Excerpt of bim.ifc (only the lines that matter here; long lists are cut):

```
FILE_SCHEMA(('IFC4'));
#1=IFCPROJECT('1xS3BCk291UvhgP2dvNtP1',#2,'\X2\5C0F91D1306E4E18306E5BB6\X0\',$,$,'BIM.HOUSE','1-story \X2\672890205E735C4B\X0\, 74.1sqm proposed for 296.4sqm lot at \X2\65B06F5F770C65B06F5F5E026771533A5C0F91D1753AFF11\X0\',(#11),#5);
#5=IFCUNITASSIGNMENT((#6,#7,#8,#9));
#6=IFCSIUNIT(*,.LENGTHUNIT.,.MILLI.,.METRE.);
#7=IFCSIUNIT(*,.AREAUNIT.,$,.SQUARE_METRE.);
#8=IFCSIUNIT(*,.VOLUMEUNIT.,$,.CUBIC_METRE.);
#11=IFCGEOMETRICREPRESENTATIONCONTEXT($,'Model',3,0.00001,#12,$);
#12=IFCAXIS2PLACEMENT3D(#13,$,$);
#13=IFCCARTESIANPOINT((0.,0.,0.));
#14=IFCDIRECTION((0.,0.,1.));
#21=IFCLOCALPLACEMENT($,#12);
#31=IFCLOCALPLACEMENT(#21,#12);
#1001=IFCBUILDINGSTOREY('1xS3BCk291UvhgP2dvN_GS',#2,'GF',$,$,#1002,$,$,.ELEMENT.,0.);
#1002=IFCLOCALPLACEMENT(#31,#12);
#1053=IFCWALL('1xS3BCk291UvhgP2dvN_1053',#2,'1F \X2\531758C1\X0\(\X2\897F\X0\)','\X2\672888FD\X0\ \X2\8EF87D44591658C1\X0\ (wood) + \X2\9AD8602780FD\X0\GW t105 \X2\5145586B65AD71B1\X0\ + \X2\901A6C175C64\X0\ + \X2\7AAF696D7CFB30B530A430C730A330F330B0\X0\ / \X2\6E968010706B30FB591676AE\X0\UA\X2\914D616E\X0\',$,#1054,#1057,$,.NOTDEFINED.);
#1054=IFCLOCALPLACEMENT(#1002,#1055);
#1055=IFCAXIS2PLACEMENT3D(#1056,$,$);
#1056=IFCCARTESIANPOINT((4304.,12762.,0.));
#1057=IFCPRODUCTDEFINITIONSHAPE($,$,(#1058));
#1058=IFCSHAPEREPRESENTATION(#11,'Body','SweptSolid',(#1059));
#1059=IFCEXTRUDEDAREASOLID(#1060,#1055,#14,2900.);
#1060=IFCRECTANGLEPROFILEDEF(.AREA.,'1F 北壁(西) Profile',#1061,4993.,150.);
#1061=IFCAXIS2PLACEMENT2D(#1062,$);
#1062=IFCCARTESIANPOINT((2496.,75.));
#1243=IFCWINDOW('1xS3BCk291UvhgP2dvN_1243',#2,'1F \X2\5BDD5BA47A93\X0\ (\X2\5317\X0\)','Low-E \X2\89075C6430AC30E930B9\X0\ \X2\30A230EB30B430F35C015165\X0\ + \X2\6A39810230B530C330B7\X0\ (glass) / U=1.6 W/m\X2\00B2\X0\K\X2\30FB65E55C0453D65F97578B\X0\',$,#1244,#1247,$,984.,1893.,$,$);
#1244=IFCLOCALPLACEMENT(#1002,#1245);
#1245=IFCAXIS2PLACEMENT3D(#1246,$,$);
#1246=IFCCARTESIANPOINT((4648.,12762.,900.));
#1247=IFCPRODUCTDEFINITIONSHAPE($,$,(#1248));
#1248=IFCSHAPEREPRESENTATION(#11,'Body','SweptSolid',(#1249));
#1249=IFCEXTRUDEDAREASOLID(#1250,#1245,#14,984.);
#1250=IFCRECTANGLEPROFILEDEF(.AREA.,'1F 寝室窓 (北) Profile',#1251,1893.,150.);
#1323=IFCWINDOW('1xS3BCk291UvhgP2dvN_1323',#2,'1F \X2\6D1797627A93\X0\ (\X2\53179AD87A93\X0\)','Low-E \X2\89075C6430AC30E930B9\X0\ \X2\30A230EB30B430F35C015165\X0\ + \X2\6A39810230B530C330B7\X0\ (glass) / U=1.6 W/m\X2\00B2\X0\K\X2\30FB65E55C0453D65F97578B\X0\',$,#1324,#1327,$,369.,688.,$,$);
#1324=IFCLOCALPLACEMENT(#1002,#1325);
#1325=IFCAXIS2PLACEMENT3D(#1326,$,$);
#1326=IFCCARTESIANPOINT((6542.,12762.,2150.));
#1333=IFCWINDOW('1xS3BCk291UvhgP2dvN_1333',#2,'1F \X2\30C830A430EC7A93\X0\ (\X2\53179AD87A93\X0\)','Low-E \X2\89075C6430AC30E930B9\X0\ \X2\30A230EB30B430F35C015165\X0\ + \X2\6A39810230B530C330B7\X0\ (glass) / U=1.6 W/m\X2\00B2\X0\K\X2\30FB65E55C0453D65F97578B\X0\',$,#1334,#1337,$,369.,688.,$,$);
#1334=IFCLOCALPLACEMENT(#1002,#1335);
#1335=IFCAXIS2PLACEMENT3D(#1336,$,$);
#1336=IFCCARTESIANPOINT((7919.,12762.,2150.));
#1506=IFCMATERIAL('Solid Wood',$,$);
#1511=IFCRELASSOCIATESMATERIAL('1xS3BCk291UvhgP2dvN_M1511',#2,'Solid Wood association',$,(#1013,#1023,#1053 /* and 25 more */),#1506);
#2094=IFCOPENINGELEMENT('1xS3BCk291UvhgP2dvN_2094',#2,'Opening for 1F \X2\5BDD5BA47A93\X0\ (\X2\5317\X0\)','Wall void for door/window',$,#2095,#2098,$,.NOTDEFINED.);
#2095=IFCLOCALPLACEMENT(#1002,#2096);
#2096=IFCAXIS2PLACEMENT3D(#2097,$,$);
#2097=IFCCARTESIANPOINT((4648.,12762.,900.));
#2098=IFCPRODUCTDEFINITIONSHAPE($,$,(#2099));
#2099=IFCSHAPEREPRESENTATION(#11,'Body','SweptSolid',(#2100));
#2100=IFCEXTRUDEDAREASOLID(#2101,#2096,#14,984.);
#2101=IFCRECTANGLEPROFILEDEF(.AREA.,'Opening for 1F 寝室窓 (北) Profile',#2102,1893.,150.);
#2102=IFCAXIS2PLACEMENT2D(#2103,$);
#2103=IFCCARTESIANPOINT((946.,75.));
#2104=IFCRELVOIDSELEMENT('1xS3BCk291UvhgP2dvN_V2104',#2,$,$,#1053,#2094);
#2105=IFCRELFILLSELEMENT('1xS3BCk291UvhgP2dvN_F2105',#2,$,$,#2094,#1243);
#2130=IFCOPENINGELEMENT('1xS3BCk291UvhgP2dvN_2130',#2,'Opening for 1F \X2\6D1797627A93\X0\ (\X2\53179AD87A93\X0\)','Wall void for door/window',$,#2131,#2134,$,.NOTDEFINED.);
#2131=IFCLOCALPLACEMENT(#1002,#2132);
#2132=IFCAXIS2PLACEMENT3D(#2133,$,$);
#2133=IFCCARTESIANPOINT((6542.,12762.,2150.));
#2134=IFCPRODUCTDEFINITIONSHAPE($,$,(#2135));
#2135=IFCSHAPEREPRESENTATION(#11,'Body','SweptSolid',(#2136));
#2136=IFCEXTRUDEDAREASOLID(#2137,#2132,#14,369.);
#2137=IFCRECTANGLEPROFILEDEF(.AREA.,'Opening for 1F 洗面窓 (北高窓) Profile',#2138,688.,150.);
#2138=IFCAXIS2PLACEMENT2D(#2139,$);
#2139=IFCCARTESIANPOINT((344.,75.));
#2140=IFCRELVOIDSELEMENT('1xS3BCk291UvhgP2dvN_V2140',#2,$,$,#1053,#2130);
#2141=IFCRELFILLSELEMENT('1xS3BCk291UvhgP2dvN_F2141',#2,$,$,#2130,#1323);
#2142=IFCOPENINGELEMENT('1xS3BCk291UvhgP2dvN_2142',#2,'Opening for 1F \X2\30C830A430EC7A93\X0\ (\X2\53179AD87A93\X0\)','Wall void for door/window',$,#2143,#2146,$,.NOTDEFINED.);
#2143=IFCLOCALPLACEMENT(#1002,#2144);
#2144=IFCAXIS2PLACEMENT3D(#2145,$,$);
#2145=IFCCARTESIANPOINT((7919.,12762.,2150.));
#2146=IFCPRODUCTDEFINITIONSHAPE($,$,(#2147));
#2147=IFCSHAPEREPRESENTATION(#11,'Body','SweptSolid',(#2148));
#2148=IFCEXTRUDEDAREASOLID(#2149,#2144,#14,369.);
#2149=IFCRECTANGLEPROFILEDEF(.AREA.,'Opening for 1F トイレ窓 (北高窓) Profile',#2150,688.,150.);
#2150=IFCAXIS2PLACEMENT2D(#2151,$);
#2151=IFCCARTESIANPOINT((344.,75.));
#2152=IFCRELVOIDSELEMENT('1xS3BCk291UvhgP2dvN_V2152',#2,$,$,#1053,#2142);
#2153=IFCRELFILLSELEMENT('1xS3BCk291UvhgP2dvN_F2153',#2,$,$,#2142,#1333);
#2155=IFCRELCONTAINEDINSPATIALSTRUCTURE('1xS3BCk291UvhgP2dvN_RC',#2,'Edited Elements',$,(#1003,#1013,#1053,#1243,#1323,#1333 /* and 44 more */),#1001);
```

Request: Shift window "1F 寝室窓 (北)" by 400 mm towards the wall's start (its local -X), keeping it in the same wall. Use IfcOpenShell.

```python
import ifcopenshell
import ifcopenshell.api.geometry
import ifcopenshell.util.placement

model = ifcopenshell.open("bim.ifc")

window = model.by_guid("1xS3BCk291UvhgP2dvN_1243")
opening = window.FillsVoids[0].RelatingOpeningElement
wall = opening.VoidsElements[0].RelatingBuildingElement

wall_matrix = ifcopenshell.util.placement.get_local_placement(wall.ObjectPlacement)
shift = wall_matrix[:3, 0] * -400.0
before = ifcopenshell.util.placement.get_local_placement(window.ObjectPlacement)[:3, 3].copy()

# The window is not placed relative to its opening, so move both.
for product in (opening, window):
    matrix = ifcopenshell.util.placement.get_local_placement(product.ObjectPlacement)
    matrix[:3, 3] += shift
    ifcopenshell.api.geometry.edit_object_placement(model, product=product, matrix=matrix, is_si=False)

after = ifcopenshell.util.placement.get_local_placement(window.ObjectPlacement)[:3, 3]
print("window moved by", (after - before).round(3) + 0.0)

model.write("bim_v2.ifc")
```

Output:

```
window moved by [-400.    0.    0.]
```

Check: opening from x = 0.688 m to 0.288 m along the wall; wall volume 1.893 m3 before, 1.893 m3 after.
